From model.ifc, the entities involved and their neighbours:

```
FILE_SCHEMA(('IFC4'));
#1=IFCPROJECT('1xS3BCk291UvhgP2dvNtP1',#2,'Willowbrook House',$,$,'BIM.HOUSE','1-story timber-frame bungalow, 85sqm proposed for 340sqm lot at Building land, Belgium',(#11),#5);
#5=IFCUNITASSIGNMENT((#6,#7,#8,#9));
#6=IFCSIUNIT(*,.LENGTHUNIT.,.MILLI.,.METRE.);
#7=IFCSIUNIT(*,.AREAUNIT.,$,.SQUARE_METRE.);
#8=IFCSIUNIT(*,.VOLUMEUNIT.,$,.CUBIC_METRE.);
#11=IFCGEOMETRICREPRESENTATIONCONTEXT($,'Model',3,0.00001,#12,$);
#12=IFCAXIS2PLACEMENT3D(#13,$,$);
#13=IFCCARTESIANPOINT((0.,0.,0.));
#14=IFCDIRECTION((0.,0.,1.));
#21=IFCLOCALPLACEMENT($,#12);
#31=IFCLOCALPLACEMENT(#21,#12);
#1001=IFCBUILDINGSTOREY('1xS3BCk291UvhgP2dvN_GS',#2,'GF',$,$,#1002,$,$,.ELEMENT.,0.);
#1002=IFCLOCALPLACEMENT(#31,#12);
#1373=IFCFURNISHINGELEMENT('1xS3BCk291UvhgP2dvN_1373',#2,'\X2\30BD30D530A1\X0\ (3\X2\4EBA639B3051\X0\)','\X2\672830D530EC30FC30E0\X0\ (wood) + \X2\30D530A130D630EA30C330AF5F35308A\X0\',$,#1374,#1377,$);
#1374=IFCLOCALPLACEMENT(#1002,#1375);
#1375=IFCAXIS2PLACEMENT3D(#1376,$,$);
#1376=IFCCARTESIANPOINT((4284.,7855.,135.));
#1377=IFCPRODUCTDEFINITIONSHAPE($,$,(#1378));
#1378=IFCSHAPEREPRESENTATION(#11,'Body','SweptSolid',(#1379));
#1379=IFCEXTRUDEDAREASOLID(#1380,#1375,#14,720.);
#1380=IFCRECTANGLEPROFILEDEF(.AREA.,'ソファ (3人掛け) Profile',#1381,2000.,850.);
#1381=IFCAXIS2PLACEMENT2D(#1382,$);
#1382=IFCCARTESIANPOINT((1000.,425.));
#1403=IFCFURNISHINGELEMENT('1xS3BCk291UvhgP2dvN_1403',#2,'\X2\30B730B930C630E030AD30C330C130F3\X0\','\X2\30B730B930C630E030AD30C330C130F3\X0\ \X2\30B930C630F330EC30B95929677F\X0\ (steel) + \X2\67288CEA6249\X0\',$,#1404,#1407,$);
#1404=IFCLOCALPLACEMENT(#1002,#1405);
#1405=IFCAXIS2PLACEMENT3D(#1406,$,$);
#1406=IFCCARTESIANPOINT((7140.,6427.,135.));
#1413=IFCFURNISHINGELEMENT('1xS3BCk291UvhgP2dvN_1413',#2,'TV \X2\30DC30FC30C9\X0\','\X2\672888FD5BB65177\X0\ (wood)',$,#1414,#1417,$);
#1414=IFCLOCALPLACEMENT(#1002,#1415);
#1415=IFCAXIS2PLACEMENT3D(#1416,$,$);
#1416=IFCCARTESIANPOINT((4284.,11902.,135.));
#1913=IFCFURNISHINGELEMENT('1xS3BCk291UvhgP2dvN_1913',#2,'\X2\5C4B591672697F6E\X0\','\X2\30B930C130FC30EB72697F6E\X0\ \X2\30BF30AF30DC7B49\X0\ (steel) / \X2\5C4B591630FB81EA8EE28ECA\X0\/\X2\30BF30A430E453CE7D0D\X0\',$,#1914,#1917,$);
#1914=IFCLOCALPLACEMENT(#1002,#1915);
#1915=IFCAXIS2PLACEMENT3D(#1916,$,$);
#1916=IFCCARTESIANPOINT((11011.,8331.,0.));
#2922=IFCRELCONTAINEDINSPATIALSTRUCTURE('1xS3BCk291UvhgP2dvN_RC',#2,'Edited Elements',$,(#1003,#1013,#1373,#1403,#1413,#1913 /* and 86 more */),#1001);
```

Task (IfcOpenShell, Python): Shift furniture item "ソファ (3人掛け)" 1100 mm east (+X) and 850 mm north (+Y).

```python
import ifcopenshell
import ifcopenshell.api.geometry
import ifcopenshell.util.placement

model = ifcopenshell.open("model.ifc")

item = model.by_guid("1xS3BCk291UvhgP2dvN_1373")
matrix = ifcopenshell.util.placement.get_local_placement(item.ObjectPlacement)
matrix[0, 3] += 1100.0
matrix[1, 3] += 850.0
ifcopenshell.api.geometry.edit_object_placement(model, product=item, matrix=matrix, is_si=False)

print(ifcopenshell.util.placement.get_local_placement(item.ObjectPlacement).round(3) + 0.0)

model.write("model-out.ifc")
```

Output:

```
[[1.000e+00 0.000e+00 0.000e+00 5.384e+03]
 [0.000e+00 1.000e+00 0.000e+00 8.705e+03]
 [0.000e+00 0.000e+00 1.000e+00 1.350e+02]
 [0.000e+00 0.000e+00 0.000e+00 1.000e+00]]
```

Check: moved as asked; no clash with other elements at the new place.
